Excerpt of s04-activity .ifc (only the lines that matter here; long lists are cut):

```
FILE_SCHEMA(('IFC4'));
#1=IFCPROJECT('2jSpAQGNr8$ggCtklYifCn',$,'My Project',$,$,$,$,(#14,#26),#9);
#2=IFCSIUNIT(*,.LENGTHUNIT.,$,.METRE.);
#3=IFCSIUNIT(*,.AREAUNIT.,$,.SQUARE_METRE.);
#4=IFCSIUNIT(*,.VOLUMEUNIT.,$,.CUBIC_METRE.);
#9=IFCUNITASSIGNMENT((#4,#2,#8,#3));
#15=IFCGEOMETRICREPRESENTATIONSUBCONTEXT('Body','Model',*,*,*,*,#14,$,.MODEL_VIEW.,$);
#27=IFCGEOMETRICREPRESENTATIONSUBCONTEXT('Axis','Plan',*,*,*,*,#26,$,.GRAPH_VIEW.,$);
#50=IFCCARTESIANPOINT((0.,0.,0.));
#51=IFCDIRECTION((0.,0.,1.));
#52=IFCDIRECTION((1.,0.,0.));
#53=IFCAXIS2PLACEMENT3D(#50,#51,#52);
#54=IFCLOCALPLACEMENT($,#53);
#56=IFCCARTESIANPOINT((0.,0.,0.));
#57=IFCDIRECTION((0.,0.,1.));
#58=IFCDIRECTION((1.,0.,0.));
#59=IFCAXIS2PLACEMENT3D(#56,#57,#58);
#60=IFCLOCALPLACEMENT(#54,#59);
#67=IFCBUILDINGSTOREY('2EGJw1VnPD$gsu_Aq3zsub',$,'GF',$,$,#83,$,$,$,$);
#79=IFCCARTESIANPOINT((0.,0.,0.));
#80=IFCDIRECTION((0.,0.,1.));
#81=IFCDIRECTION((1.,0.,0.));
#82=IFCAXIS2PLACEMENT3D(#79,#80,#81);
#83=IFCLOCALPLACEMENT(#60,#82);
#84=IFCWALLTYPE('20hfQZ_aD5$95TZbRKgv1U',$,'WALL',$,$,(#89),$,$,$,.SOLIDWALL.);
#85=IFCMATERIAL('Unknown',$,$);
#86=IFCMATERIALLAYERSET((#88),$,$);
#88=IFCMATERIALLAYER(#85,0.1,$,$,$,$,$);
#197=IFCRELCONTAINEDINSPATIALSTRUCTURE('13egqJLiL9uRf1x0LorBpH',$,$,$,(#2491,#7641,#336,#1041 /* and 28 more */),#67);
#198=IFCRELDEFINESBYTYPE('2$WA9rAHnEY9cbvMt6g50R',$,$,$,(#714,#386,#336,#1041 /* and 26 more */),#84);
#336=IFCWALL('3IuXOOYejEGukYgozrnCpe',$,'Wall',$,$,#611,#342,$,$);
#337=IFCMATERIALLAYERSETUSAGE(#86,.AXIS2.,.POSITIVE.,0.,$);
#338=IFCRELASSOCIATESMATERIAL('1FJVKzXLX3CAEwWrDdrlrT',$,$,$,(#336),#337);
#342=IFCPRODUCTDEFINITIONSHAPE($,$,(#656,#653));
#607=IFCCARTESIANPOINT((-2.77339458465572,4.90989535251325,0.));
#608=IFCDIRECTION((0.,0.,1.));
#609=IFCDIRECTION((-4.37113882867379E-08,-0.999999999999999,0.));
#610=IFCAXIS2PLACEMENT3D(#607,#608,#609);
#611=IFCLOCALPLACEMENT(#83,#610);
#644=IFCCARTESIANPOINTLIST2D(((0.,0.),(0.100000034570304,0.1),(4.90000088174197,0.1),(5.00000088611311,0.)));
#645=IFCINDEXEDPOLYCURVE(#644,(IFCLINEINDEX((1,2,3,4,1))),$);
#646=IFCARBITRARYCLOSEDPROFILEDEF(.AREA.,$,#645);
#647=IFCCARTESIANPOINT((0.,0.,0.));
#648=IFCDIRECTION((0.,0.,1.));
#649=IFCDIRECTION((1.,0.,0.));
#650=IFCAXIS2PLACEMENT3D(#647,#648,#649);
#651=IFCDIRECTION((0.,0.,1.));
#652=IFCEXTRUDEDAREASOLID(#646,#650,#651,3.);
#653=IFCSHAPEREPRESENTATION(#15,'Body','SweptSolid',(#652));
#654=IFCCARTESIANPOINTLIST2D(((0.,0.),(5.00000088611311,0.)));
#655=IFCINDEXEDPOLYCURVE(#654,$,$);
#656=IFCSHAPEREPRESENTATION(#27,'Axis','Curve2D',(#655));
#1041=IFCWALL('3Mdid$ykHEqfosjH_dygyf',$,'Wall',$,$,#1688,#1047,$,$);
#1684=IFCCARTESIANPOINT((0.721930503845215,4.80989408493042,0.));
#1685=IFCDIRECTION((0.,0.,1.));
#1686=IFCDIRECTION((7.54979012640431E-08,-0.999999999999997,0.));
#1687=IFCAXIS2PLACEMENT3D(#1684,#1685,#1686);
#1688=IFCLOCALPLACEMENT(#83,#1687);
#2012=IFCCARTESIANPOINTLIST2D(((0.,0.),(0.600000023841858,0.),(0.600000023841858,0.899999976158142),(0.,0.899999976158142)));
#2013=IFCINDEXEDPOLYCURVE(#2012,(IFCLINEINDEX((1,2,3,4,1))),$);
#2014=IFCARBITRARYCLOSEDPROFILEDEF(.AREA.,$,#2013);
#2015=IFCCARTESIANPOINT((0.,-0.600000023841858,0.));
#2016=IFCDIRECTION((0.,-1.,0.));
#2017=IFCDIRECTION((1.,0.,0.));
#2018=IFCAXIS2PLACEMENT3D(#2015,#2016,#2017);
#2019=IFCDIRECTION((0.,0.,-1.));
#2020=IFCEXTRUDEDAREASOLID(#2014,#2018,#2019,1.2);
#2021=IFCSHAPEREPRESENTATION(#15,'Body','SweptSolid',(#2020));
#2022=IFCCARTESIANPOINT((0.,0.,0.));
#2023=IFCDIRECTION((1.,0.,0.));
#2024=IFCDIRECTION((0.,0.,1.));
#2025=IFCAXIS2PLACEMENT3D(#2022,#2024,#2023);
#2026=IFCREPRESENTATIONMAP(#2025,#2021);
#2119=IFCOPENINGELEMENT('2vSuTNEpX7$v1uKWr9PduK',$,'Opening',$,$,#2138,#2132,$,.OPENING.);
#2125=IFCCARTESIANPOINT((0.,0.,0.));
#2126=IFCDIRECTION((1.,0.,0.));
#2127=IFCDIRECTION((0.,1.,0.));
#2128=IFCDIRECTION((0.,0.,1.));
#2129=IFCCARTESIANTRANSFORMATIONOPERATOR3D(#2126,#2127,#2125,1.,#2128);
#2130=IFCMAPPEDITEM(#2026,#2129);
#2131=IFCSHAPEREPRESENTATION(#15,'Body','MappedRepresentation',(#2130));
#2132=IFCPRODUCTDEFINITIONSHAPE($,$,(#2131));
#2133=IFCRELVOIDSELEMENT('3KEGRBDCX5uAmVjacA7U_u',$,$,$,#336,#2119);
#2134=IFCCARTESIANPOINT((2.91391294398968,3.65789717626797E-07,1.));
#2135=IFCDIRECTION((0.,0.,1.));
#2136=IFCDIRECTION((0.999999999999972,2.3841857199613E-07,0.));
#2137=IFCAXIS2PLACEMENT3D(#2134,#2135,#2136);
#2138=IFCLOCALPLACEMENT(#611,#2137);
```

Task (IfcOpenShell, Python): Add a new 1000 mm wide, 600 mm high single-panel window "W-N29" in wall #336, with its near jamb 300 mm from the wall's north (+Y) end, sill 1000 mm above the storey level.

```python
import numpy as np
import ifcopenshell
import ifcopenshell.api.feature
import ifcopenshell.api.geometry
import ifcopenshell.api.root
import ifcopenshell.api.spatial
import ifcopenshell.geom
import ifcopenshell.util.element
import ifcopenshell.util.placement
import ifcopenshell.util.representation
import ifcopenshell.util.shape
import ifcopenshell.util.unit

model = ifcopenshell.open("s04-activity .ifc")
unit_scale = ifcopenshell.util.unit.calculate_unit_scale(model)
settings = ifcopenshell.geom.settings()


def volume(element):
    """Net volume in cubic metres, openings subtracted."""
    shape = ifcopenshell.geom.create_shape(settings, element)
    return ifcopenshell.util.shape.get_volume(shape.geometry)


wall = model.by_id(336)
storey = ifcopenshell.util.element.get_container(wall, ifc_class="IfcBuildingStorey")
context = ifcopenshell.util.representation.get_context(model, "Model", "Body", "MODEL_VIEW")
before = volume(wall)

width, height, from_end, sill = 1, 0.6, 0.3, 1  # metres

# The wall runs along its own X axis, and the end named is its -X end.
wall_shape = ifcopenshell.geom.create_shape(settings, wall)
x, y, z = ifcopenshell.util.shape.get_vertices(wall_shape.geometry).T
start = x.min() + from_end
face, thickness = float(y.min()), float(y.max() - y.min())
wall_matrix = ifcopenshell.util.placement.get_local_placement(wall.ObjectPlacement)
level = ifcopenshell.util.placement.get_local_placement(storey.ObjectPlacement)[2, 3]


def in_wall(x, y):
    """Placement at x, y metres in the wall's axes, at sill height."""
    matrix = wall_matrix.copy()
    matrix[:, 3] = wall_matrix @ np.array([x / unit_scale, y / unit_scale, 0.0, 1.0])
    matrix[2, 3] = level + sill / unit_scale
    return matrix


# Opening: a box that overshoots both wall faces by 50 mm.
opening = ifcopenshell.api.root.create_entity(model, ifc_class="IfcOpeningElement", predefined_type="OPENING")
box = ifcopenshell.api.geometry.add_wall_representation(
    model, context=context, length=width, height=height, thickness=thickness + 0.1
)
ifcopenshell.api.geometry.assign_representation(model, product=opening, representation=box)
ifcopenshell.api.geometry.edit_object_placement(model, product=opening, matrix=in_wall(start, face - 0.05), is_si=False)
ifcopenshell.api.feature.add_feature(model, feature=opening, element=wall)

window = ifcopenshell.api.root.create_entity(model, ifc_class="IfcWindow", name="W-N29", predefined_type="WINDOW")
window.OverallWidth, window.OverallHeight = width / unit_scale, height / unit_scale
window.PartitioningType = "SINGLE_PANEL"
body = ifcopenshell.api.geometry.add_window_representation(
    model,
    context=context,
    overall_width=window.OverallWidth,
    overall_height=window.OverallHeight,
    partition_type="SINGLE_PANEL",
)
ifcopenshell.api.geometry.assign_representation(model, product=window, representation=body)
ifcopenshell.api.spatial.assign_container(model, products=[window], relating_structure=storey)
ifcopenshell.api.feature.add_filling(model, opening=opening, element=window)

# Centre the window in the wall's thickness.
ifcopenshell.api.geometry.edit_object_placement(model, product=window, matrix=in_wall(start, face), is_si=False)
window_shape = ifcopenshell.geom.create_shape(settings, window)
depth = ifcopenshell.util.shape.get_vertices(window_shape.geometry)[:, 1]
offset = face + thickness / 2 - (depth.min() + depth.max()) / 2
ifcopenshell.api.geometry.edit_object_placement(model, product=window, matrix=in_wall(start, offset), is_si=False)

after = volume(wall)

print(f"wall volume {before:.3f} -> {after:.3f} m3")

model.write("s04-activity _rev.ifc")
```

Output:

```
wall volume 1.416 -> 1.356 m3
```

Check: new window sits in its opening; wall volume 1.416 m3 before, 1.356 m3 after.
